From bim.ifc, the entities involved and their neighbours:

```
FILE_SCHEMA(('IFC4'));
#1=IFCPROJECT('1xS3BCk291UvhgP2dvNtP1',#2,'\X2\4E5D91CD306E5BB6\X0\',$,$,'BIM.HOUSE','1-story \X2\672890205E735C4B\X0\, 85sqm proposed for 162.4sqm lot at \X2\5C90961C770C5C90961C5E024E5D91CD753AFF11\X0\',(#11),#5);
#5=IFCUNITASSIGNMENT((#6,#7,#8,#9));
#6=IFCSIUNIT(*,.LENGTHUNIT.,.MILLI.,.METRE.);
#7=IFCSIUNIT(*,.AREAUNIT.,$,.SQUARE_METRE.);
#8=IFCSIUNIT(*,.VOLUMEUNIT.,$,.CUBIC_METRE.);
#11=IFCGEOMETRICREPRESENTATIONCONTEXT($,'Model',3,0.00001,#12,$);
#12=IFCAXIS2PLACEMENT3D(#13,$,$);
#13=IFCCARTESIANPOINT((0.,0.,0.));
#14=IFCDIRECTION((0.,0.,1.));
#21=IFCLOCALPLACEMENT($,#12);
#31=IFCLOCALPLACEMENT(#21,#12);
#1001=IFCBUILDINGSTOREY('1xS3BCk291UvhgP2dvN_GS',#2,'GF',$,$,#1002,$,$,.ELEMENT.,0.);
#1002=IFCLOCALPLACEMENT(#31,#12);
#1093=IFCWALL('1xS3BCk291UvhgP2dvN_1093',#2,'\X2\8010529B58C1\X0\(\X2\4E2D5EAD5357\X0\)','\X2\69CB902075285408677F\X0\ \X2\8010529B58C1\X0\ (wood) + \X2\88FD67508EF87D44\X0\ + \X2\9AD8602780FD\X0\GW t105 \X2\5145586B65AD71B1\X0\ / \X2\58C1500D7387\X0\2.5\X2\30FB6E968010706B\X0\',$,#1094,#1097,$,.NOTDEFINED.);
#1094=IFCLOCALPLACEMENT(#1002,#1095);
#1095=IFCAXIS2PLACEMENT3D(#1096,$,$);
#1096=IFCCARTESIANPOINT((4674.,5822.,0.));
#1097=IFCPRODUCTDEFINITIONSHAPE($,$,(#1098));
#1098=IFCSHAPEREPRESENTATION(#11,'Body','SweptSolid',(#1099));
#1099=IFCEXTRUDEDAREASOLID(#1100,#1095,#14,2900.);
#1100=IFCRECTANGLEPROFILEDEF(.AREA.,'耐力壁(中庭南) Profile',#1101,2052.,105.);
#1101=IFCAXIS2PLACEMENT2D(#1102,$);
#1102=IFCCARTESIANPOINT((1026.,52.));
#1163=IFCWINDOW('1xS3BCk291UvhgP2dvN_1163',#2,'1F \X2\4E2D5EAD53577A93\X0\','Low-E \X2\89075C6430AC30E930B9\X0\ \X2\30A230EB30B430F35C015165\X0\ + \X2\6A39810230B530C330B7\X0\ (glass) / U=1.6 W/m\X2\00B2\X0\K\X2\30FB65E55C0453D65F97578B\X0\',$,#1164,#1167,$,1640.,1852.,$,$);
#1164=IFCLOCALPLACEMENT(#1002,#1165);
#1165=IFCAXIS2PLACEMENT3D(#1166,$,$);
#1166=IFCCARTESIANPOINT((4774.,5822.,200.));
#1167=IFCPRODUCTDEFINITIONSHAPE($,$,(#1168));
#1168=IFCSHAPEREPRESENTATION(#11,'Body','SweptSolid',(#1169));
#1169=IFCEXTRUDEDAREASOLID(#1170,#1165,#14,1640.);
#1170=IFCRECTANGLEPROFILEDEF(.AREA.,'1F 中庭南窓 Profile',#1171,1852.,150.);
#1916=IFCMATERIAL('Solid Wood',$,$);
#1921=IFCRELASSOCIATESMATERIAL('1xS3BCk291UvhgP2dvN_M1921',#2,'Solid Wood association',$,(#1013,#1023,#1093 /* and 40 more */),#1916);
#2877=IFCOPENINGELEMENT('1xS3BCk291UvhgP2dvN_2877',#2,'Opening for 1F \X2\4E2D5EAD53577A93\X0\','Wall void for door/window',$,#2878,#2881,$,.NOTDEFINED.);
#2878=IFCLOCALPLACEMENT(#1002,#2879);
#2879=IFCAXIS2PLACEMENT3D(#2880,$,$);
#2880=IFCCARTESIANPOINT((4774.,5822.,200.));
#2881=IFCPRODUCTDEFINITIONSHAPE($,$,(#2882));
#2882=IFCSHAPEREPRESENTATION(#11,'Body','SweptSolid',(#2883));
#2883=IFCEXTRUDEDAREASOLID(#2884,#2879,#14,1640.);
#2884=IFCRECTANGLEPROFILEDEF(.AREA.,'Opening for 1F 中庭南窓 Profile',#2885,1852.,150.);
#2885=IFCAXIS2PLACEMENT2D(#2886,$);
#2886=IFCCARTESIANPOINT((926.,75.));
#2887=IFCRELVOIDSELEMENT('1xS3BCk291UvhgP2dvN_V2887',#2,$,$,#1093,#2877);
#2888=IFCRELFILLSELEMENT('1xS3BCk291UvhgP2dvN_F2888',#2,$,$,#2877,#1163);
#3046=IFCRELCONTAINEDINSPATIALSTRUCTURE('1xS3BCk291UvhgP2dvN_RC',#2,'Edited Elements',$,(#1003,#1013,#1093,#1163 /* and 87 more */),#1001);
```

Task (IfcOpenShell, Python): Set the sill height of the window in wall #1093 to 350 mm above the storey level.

```python
import numpy as np
import ifcopenshell
import ifcopenshell.api.geometry
import ifcopenshell.geom
import ifcopenshell.util.element
import ifcopenshell.util.placement
import ifcopenshell.util.shape
import ifcopenshell.util.unit

model = ifcopenshell.open("bim.ifc")
unit_scale = ifcopenshell.util.unit.calculate_unit_scale(model)

window = model.by_id(1163)
opening = window.FillsVoids[0].RelatingOpeningElement
storey = ifcopenshell.util.element.get_container(window, ifc_class="IfcBuildingStorey")
level = ifcopenshell.util.placement.get_local_placement(storey.ObjectPlacement)[2, 3]

# The opening's origin need not be at the sill, so measure its lowest point.
shape = ifcopenshell.geom.create_shape(ifcopenshell.geom.settings(), opening)
bottom = ifcopenshell.util.shape.get_shape_bottom_elevation(shape, shape.geometry) / unit_scale
dz = level + 0.35 / unit_scale - bottom

shift = np.array([0.0, 0.0, dz])
# The window is not placed relative to its opening, so move both.
for product in (opening, window):
    matrix = ifcopenshell.util.placement.get_local_placement(product.ObjectPlacement)
    matrix[:3, 3] += shift
    ifcopenshell.api.geometry.edit_object_placement(model, product=product, matrix=matrix, is_si=False)

print(f"moved by {dz * unit_scale:+.3f} m")

model.write("bim_updated.ifc")
```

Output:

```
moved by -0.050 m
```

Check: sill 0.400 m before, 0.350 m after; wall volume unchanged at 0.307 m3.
